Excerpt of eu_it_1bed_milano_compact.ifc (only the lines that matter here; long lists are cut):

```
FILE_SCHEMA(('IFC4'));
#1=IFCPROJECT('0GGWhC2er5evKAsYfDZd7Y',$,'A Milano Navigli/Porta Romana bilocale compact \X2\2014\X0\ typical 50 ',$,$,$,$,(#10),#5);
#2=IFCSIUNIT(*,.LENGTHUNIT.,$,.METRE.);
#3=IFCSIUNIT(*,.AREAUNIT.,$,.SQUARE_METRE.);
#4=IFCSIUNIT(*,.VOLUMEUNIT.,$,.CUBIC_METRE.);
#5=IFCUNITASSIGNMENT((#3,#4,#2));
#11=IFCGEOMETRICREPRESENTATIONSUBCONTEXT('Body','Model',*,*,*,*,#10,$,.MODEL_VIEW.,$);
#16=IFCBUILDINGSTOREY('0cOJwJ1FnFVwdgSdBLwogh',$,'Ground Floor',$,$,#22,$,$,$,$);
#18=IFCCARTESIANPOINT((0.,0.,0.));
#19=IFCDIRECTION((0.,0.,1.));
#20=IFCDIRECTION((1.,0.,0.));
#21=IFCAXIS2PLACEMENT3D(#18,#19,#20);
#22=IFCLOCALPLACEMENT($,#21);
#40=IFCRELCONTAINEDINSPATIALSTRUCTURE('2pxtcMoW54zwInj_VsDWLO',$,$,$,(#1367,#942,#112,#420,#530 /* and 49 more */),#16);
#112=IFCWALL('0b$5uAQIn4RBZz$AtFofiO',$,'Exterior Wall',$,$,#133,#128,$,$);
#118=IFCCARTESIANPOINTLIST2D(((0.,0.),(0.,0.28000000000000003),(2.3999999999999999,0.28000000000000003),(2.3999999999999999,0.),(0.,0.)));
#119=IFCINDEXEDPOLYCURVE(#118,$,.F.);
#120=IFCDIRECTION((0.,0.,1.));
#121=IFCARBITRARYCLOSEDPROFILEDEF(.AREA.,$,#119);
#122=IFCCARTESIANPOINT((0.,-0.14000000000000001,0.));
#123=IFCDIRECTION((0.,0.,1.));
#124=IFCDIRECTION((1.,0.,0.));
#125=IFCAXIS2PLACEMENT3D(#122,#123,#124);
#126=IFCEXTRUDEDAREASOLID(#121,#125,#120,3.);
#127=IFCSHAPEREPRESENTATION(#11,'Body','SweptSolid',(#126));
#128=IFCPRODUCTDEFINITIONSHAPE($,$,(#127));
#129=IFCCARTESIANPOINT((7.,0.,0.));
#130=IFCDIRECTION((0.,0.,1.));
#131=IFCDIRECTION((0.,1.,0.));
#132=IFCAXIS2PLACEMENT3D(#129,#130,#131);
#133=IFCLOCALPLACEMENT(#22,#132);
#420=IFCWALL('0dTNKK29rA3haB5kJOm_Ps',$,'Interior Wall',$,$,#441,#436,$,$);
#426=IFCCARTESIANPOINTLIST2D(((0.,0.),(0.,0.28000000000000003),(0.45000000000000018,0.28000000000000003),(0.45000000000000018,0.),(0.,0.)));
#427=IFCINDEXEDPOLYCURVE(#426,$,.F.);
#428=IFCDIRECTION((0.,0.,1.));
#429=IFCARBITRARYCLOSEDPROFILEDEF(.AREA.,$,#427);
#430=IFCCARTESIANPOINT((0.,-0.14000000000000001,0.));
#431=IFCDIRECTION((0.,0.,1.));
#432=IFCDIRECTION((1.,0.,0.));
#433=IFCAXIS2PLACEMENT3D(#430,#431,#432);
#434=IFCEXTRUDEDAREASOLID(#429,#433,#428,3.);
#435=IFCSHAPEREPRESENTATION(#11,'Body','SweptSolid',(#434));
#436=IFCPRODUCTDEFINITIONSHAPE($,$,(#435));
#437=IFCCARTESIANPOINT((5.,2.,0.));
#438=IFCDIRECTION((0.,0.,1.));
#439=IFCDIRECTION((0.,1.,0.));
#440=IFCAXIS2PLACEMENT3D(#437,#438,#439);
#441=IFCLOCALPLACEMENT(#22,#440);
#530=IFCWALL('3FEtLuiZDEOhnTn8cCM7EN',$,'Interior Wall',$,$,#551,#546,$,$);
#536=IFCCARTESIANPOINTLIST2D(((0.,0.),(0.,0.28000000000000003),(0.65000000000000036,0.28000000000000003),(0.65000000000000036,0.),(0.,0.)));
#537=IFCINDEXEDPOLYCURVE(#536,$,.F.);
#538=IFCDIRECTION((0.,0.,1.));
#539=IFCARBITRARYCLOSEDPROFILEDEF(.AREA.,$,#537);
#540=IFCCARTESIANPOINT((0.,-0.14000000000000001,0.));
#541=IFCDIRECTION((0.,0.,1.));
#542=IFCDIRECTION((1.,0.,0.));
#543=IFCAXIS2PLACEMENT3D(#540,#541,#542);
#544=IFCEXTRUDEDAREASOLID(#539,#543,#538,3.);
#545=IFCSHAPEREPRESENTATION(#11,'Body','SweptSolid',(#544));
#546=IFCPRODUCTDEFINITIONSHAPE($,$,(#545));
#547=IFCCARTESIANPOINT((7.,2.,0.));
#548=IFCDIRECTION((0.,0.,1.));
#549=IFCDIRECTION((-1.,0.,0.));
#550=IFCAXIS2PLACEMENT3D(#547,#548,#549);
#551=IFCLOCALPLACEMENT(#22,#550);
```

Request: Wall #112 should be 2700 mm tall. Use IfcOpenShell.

```python
import ifcopenshell
import ifcopenshell.geom
import ifcopenshell.util.representation
import ifcopenshell.util.shape
import ifcopenshell.util.unit

model = ifcopenshell.open("eu_it_1bed_milano_compact.ifc")
unit_scale = ifcopenshell.util.unit.calculate_unit_scale(model)
settings = ifcopenshell.geom.settings()


def volume(element):
    """Net volume in cubic metres, openings subtracted."""
    shape = ifcopenshell.geom.create_shape(settings, element)
    return ifcopenshell.util.shape.get_volume(shape.geometry)


wall = model.by_guid("0b$5uAQIn4RBZz$AtFofiO")
before = volume(wall)

body = ifcopenshell.util.representation.get_representation(wall, "Model", "Body")
solid = body.Items[0]
old_height = solid.Depth
solid.Depth = 2.7 / unit_scale
after = volume(wall)

print(f"height {old_height:g} -> {solid.Depth:g}, volume {before:.3f} -> {after:.3f} m3")

model.write("eu_it_1bed_milano_compact_rev.ifc")
```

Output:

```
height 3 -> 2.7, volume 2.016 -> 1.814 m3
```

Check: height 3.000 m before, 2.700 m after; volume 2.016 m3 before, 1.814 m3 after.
